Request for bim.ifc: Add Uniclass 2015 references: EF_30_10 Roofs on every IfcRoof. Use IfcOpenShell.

First a look at what the model holds.

```python
import ifcopenshell

model = ifcopenshell.open("bim.ifc")
print(model.schema)
print("classifications:", [c.Name for c in model.by_type("IfcClassification")])
for ifc_class in ("IfcDoor", "IfcRoof", "IfcStair", "IfcWall", "IfcWindow"):
    print(ifc_class, len(model.by_type(ifc_class)))
```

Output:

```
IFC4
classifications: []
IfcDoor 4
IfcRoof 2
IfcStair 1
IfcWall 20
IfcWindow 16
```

```python
import ifcopenshell
import ifcopenshell.api.classification

model = ifcopenshell.open("bim.ifc")

system = ifcopenshell.api.classification.add_classification(model, classification="Uniclass 2015")

codes = {
    "IfcRoof": ("EF_30_10", "Roofs"),
}
for ifc_class, (code, name) in codes.items():
    products = model.by_type(ifc_class)
    ifcopenshell.api.classification.add_reference(
        model, products=products, classification=system, identification=code, name=name
    )
    print(code, len(products))

model.write("bim_edited.ifc")
```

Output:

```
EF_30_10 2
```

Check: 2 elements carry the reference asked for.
